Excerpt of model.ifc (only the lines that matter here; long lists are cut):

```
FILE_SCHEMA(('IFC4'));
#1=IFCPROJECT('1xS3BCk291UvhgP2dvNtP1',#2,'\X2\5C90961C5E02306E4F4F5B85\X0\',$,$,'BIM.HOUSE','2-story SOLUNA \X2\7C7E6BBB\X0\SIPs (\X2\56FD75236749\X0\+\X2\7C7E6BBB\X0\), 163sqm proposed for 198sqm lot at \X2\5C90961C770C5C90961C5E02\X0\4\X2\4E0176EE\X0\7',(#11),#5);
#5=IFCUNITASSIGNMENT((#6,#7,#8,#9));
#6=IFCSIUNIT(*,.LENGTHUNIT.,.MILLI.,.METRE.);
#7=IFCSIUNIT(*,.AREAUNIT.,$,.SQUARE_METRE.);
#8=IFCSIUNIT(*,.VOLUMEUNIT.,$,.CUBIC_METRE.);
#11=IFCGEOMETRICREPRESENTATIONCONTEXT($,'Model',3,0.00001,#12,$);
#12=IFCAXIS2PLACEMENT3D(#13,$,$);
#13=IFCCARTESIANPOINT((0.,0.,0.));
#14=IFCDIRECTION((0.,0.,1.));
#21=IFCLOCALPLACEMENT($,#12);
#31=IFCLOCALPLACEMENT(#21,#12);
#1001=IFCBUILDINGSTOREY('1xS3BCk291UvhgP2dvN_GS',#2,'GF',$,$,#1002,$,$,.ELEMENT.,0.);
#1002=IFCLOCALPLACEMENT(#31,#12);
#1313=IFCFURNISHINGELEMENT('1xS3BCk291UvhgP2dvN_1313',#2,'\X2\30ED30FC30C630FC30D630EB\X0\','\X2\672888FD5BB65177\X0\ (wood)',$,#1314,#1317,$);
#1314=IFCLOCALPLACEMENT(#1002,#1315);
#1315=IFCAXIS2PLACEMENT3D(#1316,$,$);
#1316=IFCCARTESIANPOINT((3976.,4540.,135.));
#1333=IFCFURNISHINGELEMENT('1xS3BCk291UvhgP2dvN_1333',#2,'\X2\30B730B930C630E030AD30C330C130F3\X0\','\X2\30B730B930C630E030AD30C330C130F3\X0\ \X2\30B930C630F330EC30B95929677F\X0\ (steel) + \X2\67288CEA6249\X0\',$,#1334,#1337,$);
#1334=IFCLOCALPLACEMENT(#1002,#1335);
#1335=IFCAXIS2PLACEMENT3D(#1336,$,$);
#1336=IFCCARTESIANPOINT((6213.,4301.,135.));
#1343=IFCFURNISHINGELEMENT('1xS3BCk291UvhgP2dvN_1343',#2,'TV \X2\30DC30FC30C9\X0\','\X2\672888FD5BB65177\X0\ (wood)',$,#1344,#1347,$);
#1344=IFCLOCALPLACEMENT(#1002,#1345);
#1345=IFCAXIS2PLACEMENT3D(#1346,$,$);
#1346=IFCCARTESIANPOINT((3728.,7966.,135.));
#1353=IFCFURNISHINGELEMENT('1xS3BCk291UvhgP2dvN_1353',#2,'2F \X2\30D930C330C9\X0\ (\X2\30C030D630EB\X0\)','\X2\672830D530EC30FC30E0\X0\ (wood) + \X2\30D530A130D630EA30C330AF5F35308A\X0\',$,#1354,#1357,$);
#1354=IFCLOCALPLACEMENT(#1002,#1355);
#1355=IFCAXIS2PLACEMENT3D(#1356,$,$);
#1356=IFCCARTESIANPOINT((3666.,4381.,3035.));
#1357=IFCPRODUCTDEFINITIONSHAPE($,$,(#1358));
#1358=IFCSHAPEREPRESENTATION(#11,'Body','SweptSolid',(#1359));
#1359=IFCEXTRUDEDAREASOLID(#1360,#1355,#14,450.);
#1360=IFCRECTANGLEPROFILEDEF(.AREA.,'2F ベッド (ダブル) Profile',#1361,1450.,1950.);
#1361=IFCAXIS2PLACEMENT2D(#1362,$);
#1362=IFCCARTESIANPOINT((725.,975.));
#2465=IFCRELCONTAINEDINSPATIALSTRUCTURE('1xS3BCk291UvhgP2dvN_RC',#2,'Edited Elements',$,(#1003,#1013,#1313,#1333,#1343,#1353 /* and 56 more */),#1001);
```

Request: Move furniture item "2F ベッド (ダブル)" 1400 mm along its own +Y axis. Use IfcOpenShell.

```python
import ifcopenshell
import ifcopenshell.api.geometry
import ifcopenshell.util.placement

model = ifcopenshell.open("model.ifc")

item = model.by_guid("1xS3BCk291UvhgP2dvN_1353")
matrix = ifcopenshell.util.placement.get_local_placement(item.ObjectPlacement)
matrix[:3, 3] += matrix[:3, 1] * 1400.0
ifcopenshell.api.geometry.edit_object_placement(model, product=item, matrix=matrix, is_si=False)

print(ifcopenshell.util.placement.get_local_placement(item.ObjectPlacement).round(3) + 0.0)

model.write("model_v2.ifc")
```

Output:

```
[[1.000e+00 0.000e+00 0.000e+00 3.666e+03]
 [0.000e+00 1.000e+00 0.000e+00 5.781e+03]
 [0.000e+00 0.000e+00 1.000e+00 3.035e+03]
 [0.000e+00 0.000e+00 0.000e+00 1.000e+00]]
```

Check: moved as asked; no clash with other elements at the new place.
